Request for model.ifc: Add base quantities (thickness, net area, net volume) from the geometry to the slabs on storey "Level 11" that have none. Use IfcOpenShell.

First a look at what the model holds.

```python
import ifcopenshell
import ifcopenshell.util.element
import ifcopenshell.util.unit

model = ifcopenshell.open("model.ifc")
print(model.schema)
for unit_type in ("LENGTHUNIT", "AREAUNIT", "VOLUMEUNIT"):
    print(unit_type, ifcopenshell.util.unit.calculate_unit_scale(model, unit_type))
storey = next(s for s in model.by_type("IfcBuildingStorey") if s.Name == "Level 11")
slabs = [e for e in ifcopenshell.util.element.get_decomposition(storey) if e.is_a("IfcSlab")]
for e in sorted(slabs, key=lambda e: e.id()):
    print(e.id(), e.is_a(), e.Name, list(ifcopenshell.util.element.get_psets(e, qtos_only=True)), sep=" | ")
```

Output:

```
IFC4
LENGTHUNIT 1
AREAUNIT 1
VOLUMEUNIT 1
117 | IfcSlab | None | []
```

```python
import ifcopenshell
import ifcopenshell.api.pset
import ifcopenshell.geom
import ifcopenshell.util.element
import ifcopenshell.util.shape
import ifcopenshell.util.unit

model = ifcopenshell.open("model.ifc")
unit_scale = ifcopenshell.util.unit.calculate_unit_scale(model)
area_scale = ifcopenshell.util.unit.calculate_unit_scale(model, "AREAUNIT")
volume_scale = ifcopenshell.util.unit.calculate_unit_scale(model, "VOLUMEUNIT")
settings = ifcopenshell.geom.settings()

storey = next(s for s in model.by_type("IfcBuildingStorey") if s.Name == "Level 11")
slabs = [e for e in ifcopenshell.util.element.get_decomposition(storey) if e.is_a("IfcSlab")]

for e in sorted(slabs, key=lambda e: e.id()):
    if ifcopenshell.util.element.get_psets(e, qtos_only=True, should_inherit=False):
        continue
    # Geometry comes back in metres, in the element's own axes.
    shape = ifcopenshell.geom.create_shape(settings, e)
    values = {
        "Width": ifcopenshell.util.shape.get_z(shape.geometry) / unit_scale,
        "NetArea": ifcopenshell.util.shape.get_footprint_area(shape.geometry) / area_scale,
        "NetVolume": ifcopenshell.util.shape.get_volume(shape.geometry) / volume_scale,
    }
    qto = ifcopenshell.api.pset.add_qto(model, product=e, name="Qto_SlabBaseQuantities")
    ifcopenshell.api.pset.edit_qto(model, qto=qto, properties=values)
    print(e.id(), {k: round(v, 3) for k, v in values.items()})

model.write("model_edited.ifc")
```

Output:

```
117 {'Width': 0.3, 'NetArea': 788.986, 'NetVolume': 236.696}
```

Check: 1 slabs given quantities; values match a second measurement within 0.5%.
